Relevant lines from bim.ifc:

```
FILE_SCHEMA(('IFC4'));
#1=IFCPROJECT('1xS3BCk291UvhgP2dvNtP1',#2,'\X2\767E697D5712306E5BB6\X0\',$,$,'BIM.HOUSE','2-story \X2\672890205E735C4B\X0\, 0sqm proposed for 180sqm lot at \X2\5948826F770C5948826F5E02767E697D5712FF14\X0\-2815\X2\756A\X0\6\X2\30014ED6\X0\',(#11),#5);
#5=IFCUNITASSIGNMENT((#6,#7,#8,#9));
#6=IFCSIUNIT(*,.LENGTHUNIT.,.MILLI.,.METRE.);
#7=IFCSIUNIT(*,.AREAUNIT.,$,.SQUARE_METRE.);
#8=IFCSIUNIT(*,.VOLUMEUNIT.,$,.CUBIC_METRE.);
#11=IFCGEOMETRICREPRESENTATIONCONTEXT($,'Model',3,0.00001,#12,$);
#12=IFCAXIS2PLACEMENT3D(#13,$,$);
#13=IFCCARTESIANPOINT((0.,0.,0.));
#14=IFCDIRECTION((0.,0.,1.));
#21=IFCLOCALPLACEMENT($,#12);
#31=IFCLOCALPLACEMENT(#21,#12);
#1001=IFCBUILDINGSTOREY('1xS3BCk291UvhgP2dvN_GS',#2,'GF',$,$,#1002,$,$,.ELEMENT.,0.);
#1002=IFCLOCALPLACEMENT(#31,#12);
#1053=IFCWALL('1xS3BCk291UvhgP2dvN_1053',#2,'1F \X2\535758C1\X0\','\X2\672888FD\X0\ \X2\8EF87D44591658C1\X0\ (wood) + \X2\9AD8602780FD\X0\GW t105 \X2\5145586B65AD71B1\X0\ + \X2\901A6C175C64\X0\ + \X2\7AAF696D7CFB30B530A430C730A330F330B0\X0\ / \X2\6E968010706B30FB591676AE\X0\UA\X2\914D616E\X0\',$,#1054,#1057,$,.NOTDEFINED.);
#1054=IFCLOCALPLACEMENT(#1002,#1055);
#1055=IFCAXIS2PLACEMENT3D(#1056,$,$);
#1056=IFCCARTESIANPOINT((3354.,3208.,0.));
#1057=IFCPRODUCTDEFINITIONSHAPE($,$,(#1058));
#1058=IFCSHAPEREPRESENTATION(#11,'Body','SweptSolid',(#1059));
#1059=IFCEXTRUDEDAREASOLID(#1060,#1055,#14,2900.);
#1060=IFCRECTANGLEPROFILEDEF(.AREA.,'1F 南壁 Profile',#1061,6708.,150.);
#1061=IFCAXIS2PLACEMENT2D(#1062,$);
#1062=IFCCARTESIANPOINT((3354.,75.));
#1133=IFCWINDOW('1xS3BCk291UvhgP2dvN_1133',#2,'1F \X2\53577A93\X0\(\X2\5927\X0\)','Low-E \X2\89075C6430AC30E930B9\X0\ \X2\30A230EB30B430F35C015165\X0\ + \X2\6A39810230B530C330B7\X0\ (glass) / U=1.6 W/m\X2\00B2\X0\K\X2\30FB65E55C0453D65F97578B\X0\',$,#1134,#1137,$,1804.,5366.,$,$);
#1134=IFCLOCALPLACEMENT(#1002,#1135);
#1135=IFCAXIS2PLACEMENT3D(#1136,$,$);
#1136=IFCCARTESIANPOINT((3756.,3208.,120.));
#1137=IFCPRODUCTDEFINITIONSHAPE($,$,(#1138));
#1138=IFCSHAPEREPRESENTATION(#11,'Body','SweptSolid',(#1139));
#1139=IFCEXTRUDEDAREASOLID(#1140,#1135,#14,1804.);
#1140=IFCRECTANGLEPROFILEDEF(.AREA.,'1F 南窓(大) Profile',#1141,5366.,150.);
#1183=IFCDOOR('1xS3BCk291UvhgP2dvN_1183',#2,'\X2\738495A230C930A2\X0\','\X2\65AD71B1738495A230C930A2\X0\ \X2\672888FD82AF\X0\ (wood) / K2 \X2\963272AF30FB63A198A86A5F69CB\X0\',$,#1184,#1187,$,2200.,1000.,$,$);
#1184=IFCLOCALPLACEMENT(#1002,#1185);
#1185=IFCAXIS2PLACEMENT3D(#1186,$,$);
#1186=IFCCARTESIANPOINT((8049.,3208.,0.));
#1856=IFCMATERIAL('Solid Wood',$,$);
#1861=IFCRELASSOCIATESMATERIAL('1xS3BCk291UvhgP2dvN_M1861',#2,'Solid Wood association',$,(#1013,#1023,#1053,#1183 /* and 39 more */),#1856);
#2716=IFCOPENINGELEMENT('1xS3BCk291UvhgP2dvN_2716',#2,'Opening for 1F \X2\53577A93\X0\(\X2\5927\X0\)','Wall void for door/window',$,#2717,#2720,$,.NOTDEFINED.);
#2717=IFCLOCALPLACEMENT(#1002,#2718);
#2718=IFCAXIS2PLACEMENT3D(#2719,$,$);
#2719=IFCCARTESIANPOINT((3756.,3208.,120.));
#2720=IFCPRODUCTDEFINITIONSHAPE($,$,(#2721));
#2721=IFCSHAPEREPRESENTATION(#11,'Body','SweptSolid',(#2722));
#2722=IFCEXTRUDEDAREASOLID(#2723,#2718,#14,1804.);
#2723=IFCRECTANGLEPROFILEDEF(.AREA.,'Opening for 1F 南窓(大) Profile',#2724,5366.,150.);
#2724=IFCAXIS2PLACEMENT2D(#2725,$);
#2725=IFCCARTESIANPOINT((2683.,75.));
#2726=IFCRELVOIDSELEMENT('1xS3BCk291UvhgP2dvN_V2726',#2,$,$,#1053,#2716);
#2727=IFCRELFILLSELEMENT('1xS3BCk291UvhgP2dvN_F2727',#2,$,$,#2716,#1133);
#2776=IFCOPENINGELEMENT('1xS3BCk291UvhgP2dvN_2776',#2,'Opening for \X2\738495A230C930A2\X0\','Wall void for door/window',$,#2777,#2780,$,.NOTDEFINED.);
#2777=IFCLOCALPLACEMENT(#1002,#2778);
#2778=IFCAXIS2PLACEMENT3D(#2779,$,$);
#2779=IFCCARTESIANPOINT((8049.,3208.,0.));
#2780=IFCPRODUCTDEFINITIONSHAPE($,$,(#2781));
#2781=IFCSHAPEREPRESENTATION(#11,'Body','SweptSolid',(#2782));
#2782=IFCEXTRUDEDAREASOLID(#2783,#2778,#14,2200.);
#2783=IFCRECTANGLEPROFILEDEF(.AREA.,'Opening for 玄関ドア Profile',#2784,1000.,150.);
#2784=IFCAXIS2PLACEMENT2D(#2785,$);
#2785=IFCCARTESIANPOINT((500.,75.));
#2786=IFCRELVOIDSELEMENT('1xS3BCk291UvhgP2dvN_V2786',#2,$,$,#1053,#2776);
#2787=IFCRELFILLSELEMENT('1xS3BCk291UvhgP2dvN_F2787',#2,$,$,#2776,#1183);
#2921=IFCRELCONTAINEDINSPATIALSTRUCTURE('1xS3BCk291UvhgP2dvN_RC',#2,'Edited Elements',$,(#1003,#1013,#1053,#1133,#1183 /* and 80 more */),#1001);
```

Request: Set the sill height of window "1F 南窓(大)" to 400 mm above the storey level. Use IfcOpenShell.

```python
import numpy as np
import ifcopenshell
import ifcopenshell.api.geometry
import ifcopenshell.geom
import ifcopenshell.util.element
import ifcopenshell.util.placement
import ifcopenshell.util.shape
import ifcopenshell.util.unit

model = ifcopenshell.open("bim.ifc")
unit_scale = ifcopenshell.util.unit.calculate_unit_scale(model)

window = model.by_guid("1xS3BCk291UvhgP2dvN_1133")
opening = window.FillsVoids[0].RelatingOpeningElement
storey = ifcopenshell.util.element.get_container(window, ifc_class="IfcBuildingStorey")
level = ifcopenshell.util.placement.get_local_placement(storey.ObjectPlacement)[2, 3]

# The opening's origin need not be at the sill, so measure its lowest point.
shape = ifcopenshell.geom.create_shape(ifcopenshell.geom.settings(), opening)
bottom = ifcopenshell.util.shape.get_shape_bottom_elevation(shape, shape.geometry) / unit_scale
dz = level + 0.4 / unit_scale - bottom

shift = np.array([0.0, 0.0, dz])
# The window is not placed relative to its opening, so move both.
for product in (opening, window):
    matrix = ifcopenshell.util.placement.get_local_placement(product.ObjectPlacement)
    matrix[:3, 3] += shift
    ifcopenshell.api.geometry.edit_object_placement(model, product=product, matrix=matrix, is_si=False)

print(f"moved by {dz * unit_scale:+.3f} m")

model.write("bim-out.ifc")
```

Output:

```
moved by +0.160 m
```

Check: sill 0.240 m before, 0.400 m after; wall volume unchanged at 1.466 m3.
